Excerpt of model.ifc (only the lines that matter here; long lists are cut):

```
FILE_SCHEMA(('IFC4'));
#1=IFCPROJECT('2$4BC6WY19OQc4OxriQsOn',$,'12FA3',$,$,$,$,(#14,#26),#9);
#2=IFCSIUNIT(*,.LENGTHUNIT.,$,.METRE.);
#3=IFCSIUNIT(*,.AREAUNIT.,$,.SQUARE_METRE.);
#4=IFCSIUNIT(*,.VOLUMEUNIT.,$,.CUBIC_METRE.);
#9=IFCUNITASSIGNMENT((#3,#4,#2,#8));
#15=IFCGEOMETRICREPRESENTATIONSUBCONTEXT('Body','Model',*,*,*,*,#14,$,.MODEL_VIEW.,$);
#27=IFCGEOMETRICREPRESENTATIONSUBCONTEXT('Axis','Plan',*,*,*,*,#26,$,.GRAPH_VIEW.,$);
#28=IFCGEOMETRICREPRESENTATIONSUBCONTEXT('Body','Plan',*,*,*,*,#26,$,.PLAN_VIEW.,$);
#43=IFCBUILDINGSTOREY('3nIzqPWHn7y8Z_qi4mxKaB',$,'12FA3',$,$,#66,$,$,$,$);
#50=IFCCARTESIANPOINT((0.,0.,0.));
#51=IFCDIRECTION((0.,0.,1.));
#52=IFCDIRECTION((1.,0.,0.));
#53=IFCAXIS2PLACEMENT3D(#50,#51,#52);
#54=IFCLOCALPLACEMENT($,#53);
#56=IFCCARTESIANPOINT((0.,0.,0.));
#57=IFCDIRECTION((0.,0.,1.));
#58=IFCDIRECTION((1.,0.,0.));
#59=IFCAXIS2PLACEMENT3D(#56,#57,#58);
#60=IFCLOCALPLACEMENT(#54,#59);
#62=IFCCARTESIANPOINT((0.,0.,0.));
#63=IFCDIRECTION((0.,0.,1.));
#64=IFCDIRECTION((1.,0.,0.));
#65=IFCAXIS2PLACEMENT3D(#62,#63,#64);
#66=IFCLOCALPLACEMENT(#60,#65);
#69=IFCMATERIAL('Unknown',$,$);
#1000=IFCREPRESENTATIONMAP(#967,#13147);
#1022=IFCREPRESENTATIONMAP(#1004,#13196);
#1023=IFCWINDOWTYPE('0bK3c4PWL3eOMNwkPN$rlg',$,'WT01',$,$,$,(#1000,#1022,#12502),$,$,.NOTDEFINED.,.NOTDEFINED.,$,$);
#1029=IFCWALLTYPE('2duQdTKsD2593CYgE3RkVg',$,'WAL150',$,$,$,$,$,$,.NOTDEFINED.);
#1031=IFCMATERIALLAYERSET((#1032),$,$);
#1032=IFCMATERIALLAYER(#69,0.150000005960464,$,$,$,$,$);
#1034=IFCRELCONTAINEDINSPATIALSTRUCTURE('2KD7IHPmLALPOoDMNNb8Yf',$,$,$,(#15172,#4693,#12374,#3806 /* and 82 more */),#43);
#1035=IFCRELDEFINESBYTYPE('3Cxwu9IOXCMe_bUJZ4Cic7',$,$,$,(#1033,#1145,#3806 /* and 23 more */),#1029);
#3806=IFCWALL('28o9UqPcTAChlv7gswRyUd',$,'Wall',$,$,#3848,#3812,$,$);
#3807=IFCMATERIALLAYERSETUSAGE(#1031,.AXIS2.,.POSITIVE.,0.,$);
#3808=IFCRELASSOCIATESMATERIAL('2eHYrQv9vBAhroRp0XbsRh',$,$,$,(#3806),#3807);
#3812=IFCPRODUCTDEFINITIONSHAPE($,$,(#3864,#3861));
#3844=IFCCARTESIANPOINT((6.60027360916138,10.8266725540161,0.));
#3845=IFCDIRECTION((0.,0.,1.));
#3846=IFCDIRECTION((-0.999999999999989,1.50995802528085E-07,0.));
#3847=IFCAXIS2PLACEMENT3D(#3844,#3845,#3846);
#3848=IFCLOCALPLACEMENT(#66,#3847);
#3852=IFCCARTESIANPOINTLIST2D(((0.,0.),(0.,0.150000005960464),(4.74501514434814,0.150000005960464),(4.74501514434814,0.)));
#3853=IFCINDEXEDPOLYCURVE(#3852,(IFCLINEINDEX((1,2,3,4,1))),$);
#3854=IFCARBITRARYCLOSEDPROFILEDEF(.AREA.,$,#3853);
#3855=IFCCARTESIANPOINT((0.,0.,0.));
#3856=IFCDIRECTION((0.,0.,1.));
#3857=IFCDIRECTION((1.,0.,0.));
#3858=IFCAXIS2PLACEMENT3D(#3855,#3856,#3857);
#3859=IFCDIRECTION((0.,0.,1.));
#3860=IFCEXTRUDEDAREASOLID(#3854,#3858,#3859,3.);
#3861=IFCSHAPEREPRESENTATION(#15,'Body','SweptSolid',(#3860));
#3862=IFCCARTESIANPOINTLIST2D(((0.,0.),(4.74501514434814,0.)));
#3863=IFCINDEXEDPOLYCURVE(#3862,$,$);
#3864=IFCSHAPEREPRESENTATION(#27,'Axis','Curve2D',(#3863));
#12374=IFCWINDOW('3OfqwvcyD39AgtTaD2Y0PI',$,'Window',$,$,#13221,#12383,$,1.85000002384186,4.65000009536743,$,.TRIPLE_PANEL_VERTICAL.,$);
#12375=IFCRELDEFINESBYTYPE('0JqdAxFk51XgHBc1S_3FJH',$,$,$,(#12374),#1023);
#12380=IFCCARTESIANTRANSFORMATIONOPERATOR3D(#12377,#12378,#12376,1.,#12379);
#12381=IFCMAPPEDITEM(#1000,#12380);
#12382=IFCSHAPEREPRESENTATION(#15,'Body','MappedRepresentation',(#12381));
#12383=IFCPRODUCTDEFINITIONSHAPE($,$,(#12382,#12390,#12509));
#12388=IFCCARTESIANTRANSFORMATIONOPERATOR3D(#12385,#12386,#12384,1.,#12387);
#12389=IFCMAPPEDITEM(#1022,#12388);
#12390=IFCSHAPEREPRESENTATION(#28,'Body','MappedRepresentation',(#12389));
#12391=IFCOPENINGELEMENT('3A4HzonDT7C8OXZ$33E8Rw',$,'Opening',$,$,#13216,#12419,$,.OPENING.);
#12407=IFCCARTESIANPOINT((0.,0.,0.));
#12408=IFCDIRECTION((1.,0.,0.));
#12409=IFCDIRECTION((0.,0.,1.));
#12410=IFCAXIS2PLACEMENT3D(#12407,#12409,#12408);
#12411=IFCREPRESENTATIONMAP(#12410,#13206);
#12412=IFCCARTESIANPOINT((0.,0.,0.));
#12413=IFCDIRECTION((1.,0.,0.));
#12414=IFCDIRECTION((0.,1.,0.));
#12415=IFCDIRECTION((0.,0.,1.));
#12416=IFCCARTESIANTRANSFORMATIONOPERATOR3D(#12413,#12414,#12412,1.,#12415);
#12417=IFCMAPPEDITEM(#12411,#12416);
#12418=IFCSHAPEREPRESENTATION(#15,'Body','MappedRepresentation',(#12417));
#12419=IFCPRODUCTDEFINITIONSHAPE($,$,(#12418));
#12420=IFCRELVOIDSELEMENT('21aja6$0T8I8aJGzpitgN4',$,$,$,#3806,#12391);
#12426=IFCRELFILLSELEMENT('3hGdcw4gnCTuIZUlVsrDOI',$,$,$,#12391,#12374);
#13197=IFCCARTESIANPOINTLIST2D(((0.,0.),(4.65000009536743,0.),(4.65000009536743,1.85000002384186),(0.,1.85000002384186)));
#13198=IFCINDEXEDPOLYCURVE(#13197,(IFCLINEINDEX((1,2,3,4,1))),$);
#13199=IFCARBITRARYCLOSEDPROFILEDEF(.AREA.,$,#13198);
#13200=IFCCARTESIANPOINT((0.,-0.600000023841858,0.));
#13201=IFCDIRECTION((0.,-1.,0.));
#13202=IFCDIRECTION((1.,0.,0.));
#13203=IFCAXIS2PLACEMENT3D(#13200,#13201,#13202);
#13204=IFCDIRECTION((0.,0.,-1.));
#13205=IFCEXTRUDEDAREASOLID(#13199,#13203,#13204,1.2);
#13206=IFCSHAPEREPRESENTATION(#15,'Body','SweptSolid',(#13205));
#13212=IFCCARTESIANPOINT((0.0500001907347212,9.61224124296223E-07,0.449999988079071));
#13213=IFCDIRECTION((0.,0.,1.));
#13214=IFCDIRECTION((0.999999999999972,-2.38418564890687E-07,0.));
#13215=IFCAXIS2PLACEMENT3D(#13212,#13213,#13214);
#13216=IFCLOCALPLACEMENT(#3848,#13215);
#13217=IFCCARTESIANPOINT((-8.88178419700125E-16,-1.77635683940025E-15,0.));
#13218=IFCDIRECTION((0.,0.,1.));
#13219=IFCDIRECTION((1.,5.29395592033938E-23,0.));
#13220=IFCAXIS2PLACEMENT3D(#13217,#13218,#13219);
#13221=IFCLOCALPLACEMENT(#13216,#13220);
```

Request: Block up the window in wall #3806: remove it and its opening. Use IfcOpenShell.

```python
import ifcopenshell
import ifcopenshell.api.feature
import ifcopenshell.api.root
import ifcopenshell.geom
import ifcopenshell.util.shape

model = ifcopenshell.open("model.ifc")
settings = ifcopenshell.geom.settings()


def volume(element):
    """Net volume in cubic metres, openings subtracted."""
    shape = ifcopenshell.geom.create_shape(settings, element)
    return ifcopenshell.util.shape.get_volume(shape.geometry)


window = model.by_id(12374)
opening = window.FillsVoids[0].RelatingOpeningElement
wall = opening.VoidsElements[0].RelatingBuildingElement
before = volume(wall)

ifcopenshell.api.root.remove_product(model, product=window)
ifcopenshell.api.feature.remove_feature(model, feature=opening)

after = volume(wall)

print(f"wall volume {before:.3f} -> {after:.3f} m3")

model.write("model_rev.ifc")
```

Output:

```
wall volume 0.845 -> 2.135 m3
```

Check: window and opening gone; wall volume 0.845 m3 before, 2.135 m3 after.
